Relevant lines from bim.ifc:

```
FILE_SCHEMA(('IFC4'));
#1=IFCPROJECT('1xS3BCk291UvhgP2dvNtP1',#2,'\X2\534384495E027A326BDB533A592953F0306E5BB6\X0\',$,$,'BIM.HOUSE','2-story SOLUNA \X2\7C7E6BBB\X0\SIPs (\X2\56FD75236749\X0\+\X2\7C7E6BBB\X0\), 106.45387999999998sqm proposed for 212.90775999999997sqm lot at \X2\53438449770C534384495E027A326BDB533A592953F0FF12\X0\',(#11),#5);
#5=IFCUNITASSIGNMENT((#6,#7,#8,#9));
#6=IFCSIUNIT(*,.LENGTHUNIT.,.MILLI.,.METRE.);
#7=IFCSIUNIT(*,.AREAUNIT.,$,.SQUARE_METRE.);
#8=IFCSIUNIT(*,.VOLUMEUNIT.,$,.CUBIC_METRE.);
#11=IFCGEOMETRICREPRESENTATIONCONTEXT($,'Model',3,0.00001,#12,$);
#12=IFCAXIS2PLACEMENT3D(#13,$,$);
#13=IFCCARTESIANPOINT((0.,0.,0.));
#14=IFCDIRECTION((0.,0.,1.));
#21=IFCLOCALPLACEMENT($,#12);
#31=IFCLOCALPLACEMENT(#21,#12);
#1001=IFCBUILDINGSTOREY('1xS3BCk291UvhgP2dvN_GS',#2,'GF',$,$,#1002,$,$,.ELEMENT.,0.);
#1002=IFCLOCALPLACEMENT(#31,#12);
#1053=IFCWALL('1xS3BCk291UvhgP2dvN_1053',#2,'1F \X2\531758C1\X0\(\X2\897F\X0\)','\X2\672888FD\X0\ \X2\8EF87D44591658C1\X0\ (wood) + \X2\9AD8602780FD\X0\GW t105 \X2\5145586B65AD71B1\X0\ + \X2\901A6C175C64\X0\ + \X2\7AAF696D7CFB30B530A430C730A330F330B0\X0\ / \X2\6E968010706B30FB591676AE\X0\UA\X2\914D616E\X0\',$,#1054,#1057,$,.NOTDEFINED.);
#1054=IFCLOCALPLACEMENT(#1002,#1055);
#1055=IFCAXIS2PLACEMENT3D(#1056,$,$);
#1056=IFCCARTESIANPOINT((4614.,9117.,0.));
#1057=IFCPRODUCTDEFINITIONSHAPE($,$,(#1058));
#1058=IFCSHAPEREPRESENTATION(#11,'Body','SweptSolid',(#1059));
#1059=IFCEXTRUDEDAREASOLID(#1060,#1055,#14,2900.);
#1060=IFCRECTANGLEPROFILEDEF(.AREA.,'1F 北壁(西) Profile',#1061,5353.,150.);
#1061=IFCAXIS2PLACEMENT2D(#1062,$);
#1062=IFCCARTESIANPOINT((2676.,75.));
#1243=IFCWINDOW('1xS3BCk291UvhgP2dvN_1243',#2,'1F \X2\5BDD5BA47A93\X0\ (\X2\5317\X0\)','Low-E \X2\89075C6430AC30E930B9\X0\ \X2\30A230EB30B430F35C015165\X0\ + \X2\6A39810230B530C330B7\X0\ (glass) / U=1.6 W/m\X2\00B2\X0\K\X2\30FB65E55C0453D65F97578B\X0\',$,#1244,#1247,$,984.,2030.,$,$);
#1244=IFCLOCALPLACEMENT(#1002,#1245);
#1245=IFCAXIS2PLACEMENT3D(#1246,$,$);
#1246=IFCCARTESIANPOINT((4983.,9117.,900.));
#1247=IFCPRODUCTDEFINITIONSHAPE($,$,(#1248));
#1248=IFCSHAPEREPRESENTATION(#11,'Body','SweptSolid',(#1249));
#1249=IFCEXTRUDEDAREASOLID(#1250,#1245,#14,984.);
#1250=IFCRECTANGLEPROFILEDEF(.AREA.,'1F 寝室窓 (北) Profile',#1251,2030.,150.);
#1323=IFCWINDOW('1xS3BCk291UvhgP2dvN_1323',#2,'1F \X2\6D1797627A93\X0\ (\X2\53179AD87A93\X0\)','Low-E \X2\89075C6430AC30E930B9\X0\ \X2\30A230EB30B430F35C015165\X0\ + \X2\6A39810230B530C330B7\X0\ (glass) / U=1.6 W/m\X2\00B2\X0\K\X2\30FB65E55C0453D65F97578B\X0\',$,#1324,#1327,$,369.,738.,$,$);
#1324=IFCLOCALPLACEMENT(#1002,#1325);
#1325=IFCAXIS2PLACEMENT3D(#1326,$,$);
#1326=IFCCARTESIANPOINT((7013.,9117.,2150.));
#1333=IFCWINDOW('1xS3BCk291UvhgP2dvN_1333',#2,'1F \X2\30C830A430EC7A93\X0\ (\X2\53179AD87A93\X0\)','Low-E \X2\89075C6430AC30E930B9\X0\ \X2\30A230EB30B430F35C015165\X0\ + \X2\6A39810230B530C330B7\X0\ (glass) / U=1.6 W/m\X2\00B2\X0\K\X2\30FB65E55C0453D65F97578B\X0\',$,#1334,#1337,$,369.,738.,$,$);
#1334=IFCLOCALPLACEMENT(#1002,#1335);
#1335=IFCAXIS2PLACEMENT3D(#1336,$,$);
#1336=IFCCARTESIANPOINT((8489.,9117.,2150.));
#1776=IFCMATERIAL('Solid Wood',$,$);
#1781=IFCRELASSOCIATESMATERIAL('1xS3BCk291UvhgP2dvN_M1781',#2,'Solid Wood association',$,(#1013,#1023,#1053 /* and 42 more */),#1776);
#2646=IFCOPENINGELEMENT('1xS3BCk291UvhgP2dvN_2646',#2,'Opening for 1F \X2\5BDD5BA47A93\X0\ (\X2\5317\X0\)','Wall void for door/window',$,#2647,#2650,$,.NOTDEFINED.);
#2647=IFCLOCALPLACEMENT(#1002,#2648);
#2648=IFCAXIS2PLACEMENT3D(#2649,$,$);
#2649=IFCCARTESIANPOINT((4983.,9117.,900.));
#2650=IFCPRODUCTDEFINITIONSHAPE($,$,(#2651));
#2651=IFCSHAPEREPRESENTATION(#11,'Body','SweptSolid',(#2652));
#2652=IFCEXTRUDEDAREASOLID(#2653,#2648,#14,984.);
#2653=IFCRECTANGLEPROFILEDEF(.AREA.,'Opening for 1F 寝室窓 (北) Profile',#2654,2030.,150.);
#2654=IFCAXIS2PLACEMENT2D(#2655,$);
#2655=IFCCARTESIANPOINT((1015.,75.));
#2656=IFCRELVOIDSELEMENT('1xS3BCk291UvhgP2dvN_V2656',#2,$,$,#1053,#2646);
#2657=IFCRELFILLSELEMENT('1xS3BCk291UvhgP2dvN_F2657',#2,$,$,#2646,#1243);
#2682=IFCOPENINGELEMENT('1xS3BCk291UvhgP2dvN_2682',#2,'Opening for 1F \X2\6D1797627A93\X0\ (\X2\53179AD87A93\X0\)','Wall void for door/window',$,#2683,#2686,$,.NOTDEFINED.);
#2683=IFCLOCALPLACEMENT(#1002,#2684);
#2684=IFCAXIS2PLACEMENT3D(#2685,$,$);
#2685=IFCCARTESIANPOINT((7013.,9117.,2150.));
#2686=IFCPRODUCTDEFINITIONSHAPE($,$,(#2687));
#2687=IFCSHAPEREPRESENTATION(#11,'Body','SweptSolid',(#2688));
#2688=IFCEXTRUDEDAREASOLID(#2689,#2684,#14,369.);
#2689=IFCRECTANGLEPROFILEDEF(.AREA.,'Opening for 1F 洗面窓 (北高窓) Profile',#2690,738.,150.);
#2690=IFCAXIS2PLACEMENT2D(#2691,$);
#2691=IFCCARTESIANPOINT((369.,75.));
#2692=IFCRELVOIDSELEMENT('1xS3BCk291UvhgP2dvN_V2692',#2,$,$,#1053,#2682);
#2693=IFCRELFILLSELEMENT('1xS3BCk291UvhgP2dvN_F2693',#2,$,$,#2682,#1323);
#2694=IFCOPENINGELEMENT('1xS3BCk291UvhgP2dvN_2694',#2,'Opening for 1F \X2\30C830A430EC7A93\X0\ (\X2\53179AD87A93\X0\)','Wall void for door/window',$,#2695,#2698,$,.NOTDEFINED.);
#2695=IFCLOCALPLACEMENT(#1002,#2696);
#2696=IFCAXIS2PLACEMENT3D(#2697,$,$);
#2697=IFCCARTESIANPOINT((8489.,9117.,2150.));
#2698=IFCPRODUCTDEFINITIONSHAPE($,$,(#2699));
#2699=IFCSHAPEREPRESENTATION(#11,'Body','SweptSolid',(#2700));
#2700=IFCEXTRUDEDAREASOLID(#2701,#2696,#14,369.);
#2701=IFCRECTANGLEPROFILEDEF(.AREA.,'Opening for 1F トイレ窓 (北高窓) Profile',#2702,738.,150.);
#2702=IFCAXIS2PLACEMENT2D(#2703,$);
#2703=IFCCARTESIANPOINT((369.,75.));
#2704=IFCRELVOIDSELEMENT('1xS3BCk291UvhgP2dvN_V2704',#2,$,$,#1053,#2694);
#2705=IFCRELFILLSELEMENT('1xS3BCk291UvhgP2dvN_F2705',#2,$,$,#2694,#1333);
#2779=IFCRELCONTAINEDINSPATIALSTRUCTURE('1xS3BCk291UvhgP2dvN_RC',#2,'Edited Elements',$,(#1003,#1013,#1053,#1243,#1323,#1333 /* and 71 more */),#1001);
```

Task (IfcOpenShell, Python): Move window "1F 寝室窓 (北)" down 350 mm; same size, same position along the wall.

```python
import numpy as np
import ifcopenshell
import ifcopenshell.api.geometry
import ifcopenshell.util.placement
import ifcopenshell.util.unit

model = ifcopenshell.open("bim.ifc")
unit_scale = ifcopenshell.util.unit.calculate_unit_scale(model)

window = model.by_guid("1xS3BCk291UvhgP2dvN_1243")
opening = window.FillsVoids[0].RelatingOpeningElement
dz = -0.35 / unit_scale

shift = np.array([0.0, 0.0, dz])
# The window is not placed relative to its opening, so move both.
for product in (opening, window):
    matrix = ifcopenshell.util.placement.get_local_placement(product.ObjectPlacement)
    matrix[:3, 3] += shift
    ifcopenshell.api.geometry.edit_object_placement(model, product=product, matrix=matrix, is_si=False)

print(f"moved by {dz * unit_scale:+.3f} m")

model.write("bim_updated.ifc")
```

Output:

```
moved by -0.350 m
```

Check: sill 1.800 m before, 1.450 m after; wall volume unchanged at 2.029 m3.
